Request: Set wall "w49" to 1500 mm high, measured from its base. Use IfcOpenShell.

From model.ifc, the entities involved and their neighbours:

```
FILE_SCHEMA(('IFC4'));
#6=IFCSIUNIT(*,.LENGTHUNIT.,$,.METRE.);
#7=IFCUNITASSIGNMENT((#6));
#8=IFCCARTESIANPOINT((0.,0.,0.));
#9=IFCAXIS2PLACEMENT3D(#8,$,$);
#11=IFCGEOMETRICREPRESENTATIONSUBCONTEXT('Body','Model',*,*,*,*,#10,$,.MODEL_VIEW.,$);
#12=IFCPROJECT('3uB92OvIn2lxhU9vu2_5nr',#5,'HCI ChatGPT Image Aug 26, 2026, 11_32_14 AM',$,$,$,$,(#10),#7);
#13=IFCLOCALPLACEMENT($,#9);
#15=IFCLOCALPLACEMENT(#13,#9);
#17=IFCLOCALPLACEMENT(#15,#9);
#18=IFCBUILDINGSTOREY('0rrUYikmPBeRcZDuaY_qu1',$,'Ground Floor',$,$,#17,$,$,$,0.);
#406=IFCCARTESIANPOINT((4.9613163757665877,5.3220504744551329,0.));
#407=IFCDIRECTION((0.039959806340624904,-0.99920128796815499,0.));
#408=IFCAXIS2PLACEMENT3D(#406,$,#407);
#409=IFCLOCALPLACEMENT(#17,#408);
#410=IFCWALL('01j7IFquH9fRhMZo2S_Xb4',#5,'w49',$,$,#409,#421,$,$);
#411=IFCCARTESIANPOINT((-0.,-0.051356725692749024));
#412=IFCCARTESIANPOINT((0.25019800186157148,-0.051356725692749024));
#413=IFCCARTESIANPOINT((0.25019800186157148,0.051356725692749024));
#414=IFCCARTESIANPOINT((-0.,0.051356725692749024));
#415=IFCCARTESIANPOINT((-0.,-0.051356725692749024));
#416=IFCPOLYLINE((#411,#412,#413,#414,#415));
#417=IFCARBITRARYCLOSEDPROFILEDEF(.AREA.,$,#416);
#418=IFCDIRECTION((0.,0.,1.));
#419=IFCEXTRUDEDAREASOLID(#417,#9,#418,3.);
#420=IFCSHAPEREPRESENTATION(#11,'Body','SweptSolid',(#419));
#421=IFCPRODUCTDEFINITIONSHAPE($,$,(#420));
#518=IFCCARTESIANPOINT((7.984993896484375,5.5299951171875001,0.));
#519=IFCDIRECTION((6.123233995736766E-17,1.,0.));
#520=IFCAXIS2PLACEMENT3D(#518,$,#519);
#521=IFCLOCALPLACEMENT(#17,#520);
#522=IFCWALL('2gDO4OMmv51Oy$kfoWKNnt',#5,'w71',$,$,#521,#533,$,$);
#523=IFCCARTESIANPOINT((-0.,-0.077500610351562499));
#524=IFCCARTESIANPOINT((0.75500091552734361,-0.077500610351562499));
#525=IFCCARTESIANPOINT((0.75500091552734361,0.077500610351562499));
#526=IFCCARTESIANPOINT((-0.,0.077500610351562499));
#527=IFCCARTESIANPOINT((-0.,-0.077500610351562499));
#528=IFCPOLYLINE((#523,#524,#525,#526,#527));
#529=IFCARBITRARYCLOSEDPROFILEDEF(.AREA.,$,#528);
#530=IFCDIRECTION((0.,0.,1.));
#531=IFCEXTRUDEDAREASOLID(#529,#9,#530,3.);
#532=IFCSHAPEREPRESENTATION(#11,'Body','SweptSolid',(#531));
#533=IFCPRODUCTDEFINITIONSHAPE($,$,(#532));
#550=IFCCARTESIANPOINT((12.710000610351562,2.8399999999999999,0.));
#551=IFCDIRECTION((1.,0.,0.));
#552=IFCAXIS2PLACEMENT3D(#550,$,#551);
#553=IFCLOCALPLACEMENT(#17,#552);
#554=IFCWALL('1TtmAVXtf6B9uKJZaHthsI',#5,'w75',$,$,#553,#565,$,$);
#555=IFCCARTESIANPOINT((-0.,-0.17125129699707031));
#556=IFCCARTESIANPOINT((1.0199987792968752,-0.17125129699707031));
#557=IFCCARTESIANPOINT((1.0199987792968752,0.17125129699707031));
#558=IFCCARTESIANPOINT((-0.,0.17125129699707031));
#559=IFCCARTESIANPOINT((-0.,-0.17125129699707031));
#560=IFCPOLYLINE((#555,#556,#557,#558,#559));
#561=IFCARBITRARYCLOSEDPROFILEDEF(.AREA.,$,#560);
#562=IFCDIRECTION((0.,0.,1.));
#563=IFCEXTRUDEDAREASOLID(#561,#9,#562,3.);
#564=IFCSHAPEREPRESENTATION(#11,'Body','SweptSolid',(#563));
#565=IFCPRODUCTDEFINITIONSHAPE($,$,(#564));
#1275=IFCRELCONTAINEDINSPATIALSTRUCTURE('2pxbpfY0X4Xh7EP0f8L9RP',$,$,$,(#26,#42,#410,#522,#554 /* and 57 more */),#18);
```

```python
import ifcopenshell
import ifcopenshell.geom
import ifcopenshell.util.representation
import ifcopenshell.util.shape

model = ifcopenshell.open("model.ifc")
settings = ifcopenshell.geom.settings()


def volume(element):
    """Net volume in cubic metres, openings subtracted."""
    shape = ifcopenshell.geom.create_shape(settings, element)
    return ifcopenshell.util.shape.get_volume(shape.geometry)


wall = model.by_guid("01j7IFquH9fRhMZo2S_Xb4")
before = volume(wall)

body = ifcopenshell.util.representation.get_representation(wall, "Model", "Body")
solid = body.Items[0]
old_height = solid.Depth
solid.Depth = 1.5
after = volume(wall)

print(f"height {old_height:g} -> {solid.Depth:g}, volume {before:.3f} -> {after:.3f} m3")

model.write("model_v2.ifc")
```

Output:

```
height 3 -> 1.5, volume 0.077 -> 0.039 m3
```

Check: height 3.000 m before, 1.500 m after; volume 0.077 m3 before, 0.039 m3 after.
